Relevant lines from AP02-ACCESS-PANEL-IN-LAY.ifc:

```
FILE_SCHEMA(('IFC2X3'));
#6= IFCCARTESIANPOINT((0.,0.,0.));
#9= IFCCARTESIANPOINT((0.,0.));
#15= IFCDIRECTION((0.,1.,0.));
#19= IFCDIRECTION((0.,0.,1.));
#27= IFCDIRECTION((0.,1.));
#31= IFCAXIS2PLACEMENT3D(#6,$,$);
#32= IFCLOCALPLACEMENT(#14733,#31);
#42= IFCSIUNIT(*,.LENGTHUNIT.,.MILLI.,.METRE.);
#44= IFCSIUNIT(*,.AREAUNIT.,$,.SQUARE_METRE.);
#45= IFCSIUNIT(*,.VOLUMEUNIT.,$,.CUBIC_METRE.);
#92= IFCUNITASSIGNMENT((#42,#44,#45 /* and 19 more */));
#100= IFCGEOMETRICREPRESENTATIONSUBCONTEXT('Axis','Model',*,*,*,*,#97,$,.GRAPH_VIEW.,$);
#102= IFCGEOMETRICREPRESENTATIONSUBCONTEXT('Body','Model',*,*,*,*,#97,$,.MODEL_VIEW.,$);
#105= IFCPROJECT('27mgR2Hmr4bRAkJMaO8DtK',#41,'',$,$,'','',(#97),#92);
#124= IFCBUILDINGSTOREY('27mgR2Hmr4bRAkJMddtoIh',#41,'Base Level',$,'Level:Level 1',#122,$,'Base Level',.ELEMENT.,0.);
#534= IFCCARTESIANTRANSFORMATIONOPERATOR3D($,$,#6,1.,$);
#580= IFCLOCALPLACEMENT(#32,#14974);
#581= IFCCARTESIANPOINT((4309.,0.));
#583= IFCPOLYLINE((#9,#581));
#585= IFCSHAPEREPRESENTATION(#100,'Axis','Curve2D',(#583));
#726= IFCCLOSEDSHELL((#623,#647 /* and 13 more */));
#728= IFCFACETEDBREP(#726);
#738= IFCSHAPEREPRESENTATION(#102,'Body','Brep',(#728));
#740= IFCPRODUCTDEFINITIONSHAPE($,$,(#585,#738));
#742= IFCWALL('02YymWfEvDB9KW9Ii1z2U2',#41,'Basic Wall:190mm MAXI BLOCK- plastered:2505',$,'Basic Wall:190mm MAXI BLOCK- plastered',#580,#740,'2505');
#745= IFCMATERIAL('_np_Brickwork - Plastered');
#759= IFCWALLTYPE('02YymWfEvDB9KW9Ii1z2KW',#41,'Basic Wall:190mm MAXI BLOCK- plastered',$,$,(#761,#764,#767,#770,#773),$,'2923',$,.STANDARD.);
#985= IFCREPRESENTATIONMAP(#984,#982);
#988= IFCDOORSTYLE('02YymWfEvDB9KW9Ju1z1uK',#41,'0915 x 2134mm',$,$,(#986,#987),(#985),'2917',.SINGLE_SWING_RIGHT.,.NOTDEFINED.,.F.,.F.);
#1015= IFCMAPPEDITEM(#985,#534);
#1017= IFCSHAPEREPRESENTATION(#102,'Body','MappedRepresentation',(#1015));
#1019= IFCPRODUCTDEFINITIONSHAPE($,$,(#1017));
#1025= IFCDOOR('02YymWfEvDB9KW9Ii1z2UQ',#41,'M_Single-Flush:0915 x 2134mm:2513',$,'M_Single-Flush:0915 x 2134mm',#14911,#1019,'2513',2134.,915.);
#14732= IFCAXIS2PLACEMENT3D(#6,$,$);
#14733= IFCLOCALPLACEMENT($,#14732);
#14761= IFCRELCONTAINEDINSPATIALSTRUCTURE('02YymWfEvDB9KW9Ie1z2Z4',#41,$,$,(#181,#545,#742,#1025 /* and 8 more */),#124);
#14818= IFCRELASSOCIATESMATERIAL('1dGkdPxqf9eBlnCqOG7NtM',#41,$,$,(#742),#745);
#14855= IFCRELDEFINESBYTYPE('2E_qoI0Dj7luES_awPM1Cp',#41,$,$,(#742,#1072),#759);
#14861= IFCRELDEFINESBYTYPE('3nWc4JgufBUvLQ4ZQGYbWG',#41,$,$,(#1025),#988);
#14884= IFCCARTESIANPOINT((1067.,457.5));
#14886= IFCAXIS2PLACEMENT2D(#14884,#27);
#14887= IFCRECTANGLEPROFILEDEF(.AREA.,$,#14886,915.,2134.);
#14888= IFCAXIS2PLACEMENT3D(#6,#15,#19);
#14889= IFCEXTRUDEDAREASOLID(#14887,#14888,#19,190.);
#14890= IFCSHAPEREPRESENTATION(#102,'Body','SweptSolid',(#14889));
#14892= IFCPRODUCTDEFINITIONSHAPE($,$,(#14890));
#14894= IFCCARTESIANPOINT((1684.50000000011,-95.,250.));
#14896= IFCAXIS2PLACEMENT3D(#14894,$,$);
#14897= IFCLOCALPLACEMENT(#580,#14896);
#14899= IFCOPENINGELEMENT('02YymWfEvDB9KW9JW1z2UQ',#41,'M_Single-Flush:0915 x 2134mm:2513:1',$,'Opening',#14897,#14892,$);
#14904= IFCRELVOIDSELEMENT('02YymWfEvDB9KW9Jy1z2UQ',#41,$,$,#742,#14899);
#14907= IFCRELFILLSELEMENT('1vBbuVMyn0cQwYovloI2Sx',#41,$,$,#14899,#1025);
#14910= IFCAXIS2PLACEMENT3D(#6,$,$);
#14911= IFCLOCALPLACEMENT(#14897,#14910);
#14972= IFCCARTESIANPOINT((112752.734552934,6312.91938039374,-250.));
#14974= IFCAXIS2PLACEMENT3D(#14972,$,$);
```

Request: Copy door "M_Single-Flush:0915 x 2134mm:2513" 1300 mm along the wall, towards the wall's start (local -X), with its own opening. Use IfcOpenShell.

```python
import ifcopenshell
import ifcopenshell.api.feature
import ifcopenshell.api.geometry
import ifcopenshell.api.root
import ifcopenshell.geom
import ifcopenshell.util.element
import ifcopenshell.util.placement
import ifcopenshell.util.shape
import ifcopenshell.util.unit

model = ifcopenshell.open("AP02-ACCESS-PANEL-IN-LAY.ifc")
unit_scale = ifcopenshell.util.unit.calculate_unit_scale(model)
settings = ifcopenshell.geom.settings()


def volume(element):
    """Net volume in cubic metres, openings subtracted."""
    shape = ifcopenshell.geom.create_shape(settings, element)
    return ifcopenshell.util.shape.get_volume(shape.geometry)


def reuse_history(source, copy):
    """copy_class also copies each property set's owner history, people and application; keep the originals."""
    for rel in copy.IsDefinedBy:
        if rel.is_a("IfcRelDefinesByProperties") and (history := rel.RelatingPropertyDefinition.OwnerHistory):
            rel.RelatingPropertyDefinition.OwnerHistory = source.OwnerHistory
            ifcopenshell.util.element.remove_deep2(model, history)


door = model.by_guid("02YymWfEvDB9KW9Ii1z2UQ")
opening = door.FillsVoids[0].RelatingOpeningElement
wall = opening.VoidsElements[0].RelatingBuildingElement
before = volume(wall)
shift = ifcopenshell.util.placement.get_local_placement(wall.ObjectPlacement)[:3, 0] * -1.3 / unit_scale

# copy_class copies the void relationship, type, container and properties, but no geometry.
new_opening = ifcopenshell.api.root.copy_class(model, product=opening)
new_opening.Representation = ifcopenshell.util.element.copy_deep(
    model, opening.Representation, exclude=["IfcGeometricRepresentationContext", "IfcRepresentationMap"]
)
new_opening.Name = "M_Single-Flush:0915 x 2134mm"
new_door = ifcopenshell.api.root.copy_class(model, product=door)
new_door.Representation = ifcopenshell.util.element.copy_deep(
    model, door.Representation, exclude=["IfcGeometricRepresentationContext", "IfcRepresentationMap"]
)
new_door.Name = "M_Single-Flush:0915 x 2134mm"
new_door.Tag = None
reuse_history(door, new_door)
fills = ifcopenshell.api.feature.add_filling(model, opening=new_opening, element=new_door)
fills.OwnerHistory = new_door.OwnerHistory  # required in IFC2X3

for old, new in ((opening, new_opening), (door, new_door)):
    matrix = ifcopenshell.util.placement.get_local_placement(old.ObjectPlacement)
    matrix[:3, 3] += shift
    ifcopenshell.api.geometry.edit_object_placement(model, product=new, matrix=matrix, is_si=False)

after = volume(wall)

print(f"wall volume {before:.3f} -> {after:.3f} m3")

model.write("AP02-ACCESS-PANEL-IN-LAY_v2.ifc")
```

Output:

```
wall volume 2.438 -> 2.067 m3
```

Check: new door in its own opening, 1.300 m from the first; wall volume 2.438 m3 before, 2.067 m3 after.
